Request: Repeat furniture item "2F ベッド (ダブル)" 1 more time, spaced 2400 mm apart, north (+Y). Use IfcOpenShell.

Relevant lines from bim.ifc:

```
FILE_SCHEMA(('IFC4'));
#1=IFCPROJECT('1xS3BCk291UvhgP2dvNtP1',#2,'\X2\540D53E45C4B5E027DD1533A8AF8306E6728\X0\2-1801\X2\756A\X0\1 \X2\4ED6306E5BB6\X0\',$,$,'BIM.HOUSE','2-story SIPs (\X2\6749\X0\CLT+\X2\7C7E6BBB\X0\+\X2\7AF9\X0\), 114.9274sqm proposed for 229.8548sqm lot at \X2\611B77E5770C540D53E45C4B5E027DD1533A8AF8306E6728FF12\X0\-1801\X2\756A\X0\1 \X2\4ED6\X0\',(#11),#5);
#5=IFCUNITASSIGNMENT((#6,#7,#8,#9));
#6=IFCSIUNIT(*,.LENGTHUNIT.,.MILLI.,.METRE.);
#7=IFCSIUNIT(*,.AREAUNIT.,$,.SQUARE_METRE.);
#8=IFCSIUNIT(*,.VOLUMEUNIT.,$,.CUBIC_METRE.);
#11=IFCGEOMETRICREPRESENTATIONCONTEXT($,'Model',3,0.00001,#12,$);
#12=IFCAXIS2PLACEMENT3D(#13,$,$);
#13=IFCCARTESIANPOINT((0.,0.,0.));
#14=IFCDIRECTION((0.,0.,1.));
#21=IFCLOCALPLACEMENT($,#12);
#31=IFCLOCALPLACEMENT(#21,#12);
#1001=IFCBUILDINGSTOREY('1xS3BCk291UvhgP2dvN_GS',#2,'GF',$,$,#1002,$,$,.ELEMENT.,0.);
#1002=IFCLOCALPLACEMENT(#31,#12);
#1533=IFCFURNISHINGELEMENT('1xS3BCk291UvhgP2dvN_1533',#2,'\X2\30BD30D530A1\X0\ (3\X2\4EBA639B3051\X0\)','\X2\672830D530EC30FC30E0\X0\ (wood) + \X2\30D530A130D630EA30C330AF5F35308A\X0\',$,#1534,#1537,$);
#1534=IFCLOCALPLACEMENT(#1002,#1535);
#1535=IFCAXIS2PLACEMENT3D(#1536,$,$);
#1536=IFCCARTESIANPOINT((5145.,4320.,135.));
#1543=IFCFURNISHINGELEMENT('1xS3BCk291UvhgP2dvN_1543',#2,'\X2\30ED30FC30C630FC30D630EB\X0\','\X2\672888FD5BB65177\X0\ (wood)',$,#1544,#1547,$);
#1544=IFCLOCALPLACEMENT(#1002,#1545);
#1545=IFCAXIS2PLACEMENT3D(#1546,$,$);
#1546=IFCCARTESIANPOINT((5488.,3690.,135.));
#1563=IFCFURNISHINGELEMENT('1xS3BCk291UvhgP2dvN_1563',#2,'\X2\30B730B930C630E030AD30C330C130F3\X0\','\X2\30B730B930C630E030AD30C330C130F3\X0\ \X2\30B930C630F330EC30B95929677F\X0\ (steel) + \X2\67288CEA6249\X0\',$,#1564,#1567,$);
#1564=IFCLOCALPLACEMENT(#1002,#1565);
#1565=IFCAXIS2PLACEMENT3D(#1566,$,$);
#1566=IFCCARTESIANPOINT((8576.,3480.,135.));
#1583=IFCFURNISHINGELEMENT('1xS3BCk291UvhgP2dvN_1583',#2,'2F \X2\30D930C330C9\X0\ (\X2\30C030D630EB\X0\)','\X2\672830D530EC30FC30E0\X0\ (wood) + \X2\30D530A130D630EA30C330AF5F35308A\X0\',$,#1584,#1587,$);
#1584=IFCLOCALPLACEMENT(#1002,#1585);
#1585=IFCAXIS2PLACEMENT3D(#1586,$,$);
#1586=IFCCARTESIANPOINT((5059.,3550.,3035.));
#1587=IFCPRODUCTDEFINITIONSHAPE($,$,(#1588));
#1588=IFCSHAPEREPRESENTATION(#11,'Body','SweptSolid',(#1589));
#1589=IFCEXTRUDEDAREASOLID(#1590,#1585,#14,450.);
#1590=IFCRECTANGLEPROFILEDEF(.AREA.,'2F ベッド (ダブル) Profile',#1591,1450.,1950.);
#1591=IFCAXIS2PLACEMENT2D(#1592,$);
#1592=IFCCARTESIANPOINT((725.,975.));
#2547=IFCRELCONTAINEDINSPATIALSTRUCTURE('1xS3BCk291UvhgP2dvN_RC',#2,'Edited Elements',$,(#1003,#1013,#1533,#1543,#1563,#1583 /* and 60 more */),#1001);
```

```python
import numpy as np
import ifcopenshell
import ifcopenshell.api.geometry
import ifcopenshell.api.root
import ifcopenshell.util.element
import ifcopenshell.util.placement
import ifcopenshell.util.unit

model = ifcopenshell.open("bim.ifc")
unit_scale = ifcopenshell.util.unit.calculate_unit_scale(model)


def reuse_history(source, copy):
    """copy_class also copies each property set's owner history, people and application; keep the originals."""
    for rel in copy.IsDefinedBy:
        if rel.is_a("IfcRelDefinesByProperties") and (history := rel.RelatingPropertyDefinition.OwnerHistory):
            rel.RelatingPropertyDefinition.OwnerHistory = source.OwnerHistory
            ifcopenshell.util.element.remove_deep2(model, history)


source = model.by_guid("1xS3BCk291UvhgP2dvN_1583")
base = ifcopenshell.util.placement.get_local_placement(source.ObjectPlacement)
step = np.array([0.0, 1.0, 0.0]) * 2.4 / unit_scale

for i in range(1, 2):
    copy = ifcopenshell.api.root.copy_class(model, product=source)
    copy.Representation = ifcopenshell.util.element.copy_deep(
        model, source.Representation, exclude=["IfcGeometricRepresentationContext", "IfcRepresentationMap"]
    )
    reuse_history(source, copy)
    matrix = base.copy()
    matrix[:3, 3] += i * step
    print("added at", matrix[:3, 3].round(3) + 0.0)
    ifcopenshell.api.geometry.edit_object_placement(model, product=copy, matrix=matrix, is_si=False)

model.write("bim_edited.ifc")
```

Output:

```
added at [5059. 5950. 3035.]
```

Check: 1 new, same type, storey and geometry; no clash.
